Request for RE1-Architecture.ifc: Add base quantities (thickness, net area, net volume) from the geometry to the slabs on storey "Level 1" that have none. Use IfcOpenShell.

First a look at what the model holds.

```python
import ifcopenshell
import ifcopenshell.util.element
import ifcopenshell.util.unit

model = ifcopenshell.open("RE1-Architecture.ifc")
print(model.schema)
for unit_type in ("LENGTHUNIT", "AREAUNIT", "VOLUMEUNIT"):
    print(unit_type, ifcopenshell.util.unit.calculate_unit_scale(model, unit_type))
storey = next(s for s in model.by_type("IfcBuildingStorey") if s.Name == "Level 1")
slabs = [e for e in ifcopenshell.util.element.get_decomposition(storey) if e.is_a("IfcSlab")]
for e in sorted(slabs, key=lambda e: e.id()):
    print(e.id(), e.is_a(), e.Name, list(ifcopenshell.util.element.get_psets(e, qtos_only=True)), sep=" | ")
```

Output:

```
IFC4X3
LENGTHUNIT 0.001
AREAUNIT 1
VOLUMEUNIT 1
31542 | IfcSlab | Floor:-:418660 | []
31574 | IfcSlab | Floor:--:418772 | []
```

```python
import ifcopenshell
import ifcopenshell.api.pset
import ifcopenshell.geom
import ifcopenshell.util.element
import ifcopenshell.util.shape
import ifcopenshell.util.unit

model = ifcopenshell.open("RE1-Architecture.ifc")
unit_scale = ifcopenshell.util.unit.calculate_unit_scale(model)
area_scale = ifcopenshell.util.unit.calculate_unit_scale(model, "AREAUNIT")
volume_scale = ifcopenshell.util.unit.calculate_unit_scale(model, "VOLUMEUNIT")
settings = ifcopenshell.geom.settings()

storey = next(s for s in model.by_type("IfcBuildingStorey") if s.Name == "Level 1")
slabs = [e for e in ifcopenshell.util.element.get_decomposition(storey) if e.is_a("IfcSlab")]

for e in sorted(slabs, key=lambda e: e.id()):
    if ifcopenshell.util.element.get_psets(e, qtos_only=True, should_inherit=False):
        continue
    # Geometry comes back in metres, in the element's own axes.
    shape = ifcopenshell.geom.create_shape(settings, e)
    values = {
        "Width": ifcopenshell.util.shape.get_z(shape.geometry) / unit_scale,
        "NetArea": ifcopenshell.util.shape.get_footprint_area(shape.geometry) / area_scale,
        "NetVolume": ifcopenshell.util.shape.get_volume(shape.geometry) / volume_scale,
    }
    qto = ifcopenshell.api.pset.add_qto(model, product=e, name="Qto_SlabBaseQuantities")
    ifcopenshell.api.pset.edit_qto(model, qto=qto, properties=values)
    print(e.id(), {k: round(v, 3) for k, v in values.items()})

model.write("RE1-Architecture_edited.ifc")
```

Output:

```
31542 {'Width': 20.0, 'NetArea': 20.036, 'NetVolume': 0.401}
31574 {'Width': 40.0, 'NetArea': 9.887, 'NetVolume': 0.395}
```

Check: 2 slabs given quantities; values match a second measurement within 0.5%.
